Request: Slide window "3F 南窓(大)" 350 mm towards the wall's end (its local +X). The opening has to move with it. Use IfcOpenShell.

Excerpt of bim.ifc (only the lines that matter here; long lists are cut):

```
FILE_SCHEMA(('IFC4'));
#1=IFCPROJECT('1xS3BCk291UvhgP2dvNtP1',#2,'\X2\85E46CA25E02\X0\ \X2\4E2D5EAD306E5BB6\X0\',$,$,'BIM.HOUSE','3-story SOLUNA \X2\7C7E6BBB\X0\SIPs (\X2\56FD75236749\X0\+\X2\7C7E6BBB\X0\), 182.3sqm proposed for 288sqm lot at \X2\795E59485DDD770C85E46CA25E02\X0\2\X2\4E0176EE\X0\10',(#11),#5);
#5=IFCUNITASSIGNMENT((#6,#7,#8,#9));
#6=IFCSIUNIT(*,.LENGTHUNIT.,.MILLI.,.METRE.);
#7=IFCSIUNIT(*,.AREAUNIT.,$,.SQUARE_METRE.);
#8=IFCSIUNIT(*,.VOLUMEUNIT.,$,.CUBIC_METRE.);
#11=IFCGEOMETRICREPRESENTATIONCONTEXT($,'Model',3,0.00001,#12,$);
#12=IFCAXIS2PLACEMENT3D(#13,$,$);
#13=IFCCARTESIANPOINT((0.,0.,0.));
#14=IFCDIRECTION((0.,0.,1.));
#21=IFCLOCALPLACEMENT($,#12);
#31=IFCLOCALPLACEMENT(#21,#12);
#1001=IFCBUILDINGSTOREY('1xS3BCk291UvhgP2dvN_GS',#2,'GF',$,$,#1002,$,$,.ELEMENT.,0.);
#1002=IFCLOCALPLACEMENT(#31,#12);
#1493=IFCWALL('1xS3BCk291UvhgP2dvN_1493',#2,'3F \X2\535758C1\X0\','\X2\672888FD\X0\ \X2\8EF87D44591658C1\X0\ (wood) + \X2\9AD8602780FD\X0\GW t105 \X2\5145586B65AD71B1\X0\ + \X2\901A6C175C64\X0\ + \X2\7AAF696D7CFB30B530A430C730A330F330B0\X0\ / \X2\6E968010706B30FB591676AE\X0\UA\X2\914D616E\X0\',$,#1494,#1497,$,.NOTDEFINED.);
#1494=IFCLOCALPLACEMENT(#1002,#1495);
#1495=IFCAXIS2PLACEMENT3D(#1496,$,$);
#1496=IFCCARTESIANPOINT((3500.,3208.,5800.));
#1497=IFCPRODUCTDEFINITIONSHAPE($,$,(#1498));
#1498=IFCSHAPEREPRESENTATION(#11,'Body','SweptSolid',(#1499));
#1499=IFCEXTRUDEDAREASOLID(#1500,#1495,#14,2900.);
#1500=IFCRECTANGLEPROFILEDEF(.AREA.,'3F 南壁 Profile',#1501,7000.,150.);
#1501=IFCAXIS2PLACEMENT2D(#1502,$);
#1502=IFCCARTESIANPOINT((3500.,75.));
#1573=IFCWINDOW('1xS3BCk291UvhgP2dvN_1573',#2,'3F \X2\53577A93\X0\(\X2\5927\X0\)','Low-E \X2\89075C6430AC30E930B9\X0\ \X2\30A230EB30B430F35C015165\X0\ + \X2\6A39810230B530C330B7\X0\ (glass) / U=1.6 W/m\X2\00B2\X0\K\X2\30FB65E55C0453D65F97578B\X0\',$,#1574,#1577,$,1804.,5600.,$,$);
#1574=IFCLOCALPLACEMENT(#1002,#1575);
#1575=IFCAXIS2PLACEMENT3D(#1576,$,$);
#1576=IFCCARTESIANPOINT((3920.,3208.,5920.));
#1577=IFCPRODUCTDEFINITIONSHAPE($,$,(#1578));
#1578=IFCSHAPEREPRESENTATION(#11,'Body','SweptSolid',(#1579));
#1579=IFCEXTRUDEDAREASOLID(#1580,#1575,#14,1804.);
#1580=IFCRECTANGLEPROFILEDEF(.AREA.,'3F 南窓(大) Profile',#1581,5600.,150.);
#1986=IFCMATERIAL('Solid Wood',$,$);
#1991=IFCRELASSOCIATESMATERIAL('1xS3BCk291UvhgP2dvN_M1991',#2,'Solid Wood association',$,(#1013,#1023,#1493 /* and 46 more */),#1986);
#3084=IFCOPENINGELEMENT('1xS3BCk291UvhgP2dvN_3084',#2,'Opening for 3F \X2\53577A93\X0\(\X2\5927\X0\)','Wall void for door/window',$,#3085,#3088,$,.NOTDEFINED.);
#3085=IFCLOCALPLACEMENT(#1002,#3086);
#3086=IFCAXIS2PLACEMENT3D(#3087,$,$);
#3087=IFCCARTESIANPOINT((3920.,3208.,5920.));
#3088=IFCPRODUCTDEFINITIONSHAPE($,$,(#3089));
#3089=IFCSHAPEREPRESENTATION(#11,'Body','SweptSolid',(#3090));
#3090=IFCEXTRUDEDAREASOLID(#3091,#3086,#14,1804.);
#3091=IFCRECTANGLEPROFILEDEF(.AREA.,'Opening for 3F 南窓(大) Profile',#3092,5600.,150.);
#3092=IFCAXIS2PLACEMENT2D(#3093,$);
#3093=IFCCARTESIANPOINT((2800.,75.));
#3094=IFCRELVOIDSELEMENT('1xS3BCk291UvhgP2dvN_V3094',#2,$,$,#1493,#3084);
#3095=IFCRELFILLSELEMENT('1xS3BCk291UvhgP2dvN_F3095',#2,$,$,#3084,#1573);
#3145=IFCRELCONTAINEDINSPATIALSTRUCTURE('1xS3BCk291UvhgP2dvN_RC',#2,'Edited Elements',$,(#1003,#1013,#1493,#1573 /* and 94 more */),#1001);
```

```python
import ifcopenshell
import ifcopenshell.api.geometry
import ifcopenshell.util.placement
import ifcopenshell.util.unit

model = ifcopenshell.open("bim.ifc")
unit_scale = ifcopenshell.util.unit.calculate_unit_scale(model)

window = model.by_id(1573)
opening = window.FillsVoids[0].RelatingOpeningElement
wall = opening.VoidsElements[0].RelatingBuildingElement

wall_matrix = ifcopenshell.util.placement.get_local_placement(wall.ObjectPlacement)
shift = wall_matrix[:3, 0] * 0.35 / unit_scale
before = ifcopenshell.util.placement.get_local_placement(window.ObjectPlacement)[:3, 3].copy()

# The window is not placed relative to its opening, so move both.
for product in (opening, window):
    matrix = ifcopenshell.util.placement.get_local_placement(product.ObjectPlacement)
    matrix[:3, 3] += shift
    ifcopenshell.api.geometry.edit_object_placement(model, product=product, matrix=matrix, is_si=False)

after = ifcopenshell.util.placement.get_local_placement(window.ObjectPlacement)[:3, 3]
print("window moved by", (after - before).round(3) + 0.0)

model.write("bim_v2.ifc")
```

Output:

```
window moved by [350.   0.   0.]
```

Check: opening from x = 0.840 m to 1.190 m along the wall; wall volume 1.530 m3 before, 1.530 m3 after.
